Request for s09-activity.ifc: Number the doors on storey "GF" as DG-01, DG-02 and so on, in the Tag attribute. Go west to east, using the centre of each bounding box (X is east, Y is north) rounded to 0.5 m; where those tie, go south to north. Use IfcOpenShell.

First a look at what the model holds.

```python
import ifcopenshell
import ifcopenshell.util.element
import ifcopenshell.util.placement

model = ifcopenshell.open("s09-activity.ifc")
print(model.schema)
storey = next(s for s in model.by_type("IfcBuildingStorey") if s.Name == "GF")
doors = [e for e in ifcopenshell.util.element.get_decomposition(storey) if e.is_a("IfcDoor")]
for e in sorted(doors, key=lambda e: e.id()):
    origin = ifcopenshell.util.placement.get_local_placement(e.ObjectPlacement)[:3, 3]
    print(e.id(), e.Tag, e.Name, origin.round(2) + 0.0, sep=" | ")
```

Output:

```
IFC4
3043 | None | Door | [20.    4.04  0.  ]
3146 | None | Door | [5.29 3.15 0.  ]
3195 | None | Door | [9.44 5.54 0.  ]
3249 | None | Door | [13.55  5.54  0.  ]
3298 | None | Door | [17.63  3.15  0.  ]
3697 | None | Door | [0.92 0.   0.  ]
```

```python
import ifcopenshell
import ifcopenshell.geom
import ifcopenshell.util.element
import ifcopenshell.util.shape

model = ifcopenshell.open("s09-activity.ifc")
settings = ifcopenshell.geom.settings()
settings.set("use-world-coords", True)


def centre(element):
    shape = ifcopenshell.geom.create_shape(settings, element)
    return ifcopenshell.util.shape.get_bbox_centroid(shape.geometry)


storey = next(s for s in model.by_type("IfcBuildingStorey") if s.Name == "GF")
doors = [e for e in ifcopenshell.util.element.get_decomposition(storey) if e.is_a("IfcDoor")]

# Insertion points can sit at a corner or the storey origin, so sort by the geometry (in metres).
centres = {e: centre(e) for e in doors}
doors.sort(key=lambda e: (round(centres[e][0] / 0.5), centres[e][1]))

for i, e in enumerate(doors, start=1):
    number = f"DG-{i:02d}"
    e.Tag = number
    print(e.id(), number)

model.write("s09-activity_updated.ifc")
```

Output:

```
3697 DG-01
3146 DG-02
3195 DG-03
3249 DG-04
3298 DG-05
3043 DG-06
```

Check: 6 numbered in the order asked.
